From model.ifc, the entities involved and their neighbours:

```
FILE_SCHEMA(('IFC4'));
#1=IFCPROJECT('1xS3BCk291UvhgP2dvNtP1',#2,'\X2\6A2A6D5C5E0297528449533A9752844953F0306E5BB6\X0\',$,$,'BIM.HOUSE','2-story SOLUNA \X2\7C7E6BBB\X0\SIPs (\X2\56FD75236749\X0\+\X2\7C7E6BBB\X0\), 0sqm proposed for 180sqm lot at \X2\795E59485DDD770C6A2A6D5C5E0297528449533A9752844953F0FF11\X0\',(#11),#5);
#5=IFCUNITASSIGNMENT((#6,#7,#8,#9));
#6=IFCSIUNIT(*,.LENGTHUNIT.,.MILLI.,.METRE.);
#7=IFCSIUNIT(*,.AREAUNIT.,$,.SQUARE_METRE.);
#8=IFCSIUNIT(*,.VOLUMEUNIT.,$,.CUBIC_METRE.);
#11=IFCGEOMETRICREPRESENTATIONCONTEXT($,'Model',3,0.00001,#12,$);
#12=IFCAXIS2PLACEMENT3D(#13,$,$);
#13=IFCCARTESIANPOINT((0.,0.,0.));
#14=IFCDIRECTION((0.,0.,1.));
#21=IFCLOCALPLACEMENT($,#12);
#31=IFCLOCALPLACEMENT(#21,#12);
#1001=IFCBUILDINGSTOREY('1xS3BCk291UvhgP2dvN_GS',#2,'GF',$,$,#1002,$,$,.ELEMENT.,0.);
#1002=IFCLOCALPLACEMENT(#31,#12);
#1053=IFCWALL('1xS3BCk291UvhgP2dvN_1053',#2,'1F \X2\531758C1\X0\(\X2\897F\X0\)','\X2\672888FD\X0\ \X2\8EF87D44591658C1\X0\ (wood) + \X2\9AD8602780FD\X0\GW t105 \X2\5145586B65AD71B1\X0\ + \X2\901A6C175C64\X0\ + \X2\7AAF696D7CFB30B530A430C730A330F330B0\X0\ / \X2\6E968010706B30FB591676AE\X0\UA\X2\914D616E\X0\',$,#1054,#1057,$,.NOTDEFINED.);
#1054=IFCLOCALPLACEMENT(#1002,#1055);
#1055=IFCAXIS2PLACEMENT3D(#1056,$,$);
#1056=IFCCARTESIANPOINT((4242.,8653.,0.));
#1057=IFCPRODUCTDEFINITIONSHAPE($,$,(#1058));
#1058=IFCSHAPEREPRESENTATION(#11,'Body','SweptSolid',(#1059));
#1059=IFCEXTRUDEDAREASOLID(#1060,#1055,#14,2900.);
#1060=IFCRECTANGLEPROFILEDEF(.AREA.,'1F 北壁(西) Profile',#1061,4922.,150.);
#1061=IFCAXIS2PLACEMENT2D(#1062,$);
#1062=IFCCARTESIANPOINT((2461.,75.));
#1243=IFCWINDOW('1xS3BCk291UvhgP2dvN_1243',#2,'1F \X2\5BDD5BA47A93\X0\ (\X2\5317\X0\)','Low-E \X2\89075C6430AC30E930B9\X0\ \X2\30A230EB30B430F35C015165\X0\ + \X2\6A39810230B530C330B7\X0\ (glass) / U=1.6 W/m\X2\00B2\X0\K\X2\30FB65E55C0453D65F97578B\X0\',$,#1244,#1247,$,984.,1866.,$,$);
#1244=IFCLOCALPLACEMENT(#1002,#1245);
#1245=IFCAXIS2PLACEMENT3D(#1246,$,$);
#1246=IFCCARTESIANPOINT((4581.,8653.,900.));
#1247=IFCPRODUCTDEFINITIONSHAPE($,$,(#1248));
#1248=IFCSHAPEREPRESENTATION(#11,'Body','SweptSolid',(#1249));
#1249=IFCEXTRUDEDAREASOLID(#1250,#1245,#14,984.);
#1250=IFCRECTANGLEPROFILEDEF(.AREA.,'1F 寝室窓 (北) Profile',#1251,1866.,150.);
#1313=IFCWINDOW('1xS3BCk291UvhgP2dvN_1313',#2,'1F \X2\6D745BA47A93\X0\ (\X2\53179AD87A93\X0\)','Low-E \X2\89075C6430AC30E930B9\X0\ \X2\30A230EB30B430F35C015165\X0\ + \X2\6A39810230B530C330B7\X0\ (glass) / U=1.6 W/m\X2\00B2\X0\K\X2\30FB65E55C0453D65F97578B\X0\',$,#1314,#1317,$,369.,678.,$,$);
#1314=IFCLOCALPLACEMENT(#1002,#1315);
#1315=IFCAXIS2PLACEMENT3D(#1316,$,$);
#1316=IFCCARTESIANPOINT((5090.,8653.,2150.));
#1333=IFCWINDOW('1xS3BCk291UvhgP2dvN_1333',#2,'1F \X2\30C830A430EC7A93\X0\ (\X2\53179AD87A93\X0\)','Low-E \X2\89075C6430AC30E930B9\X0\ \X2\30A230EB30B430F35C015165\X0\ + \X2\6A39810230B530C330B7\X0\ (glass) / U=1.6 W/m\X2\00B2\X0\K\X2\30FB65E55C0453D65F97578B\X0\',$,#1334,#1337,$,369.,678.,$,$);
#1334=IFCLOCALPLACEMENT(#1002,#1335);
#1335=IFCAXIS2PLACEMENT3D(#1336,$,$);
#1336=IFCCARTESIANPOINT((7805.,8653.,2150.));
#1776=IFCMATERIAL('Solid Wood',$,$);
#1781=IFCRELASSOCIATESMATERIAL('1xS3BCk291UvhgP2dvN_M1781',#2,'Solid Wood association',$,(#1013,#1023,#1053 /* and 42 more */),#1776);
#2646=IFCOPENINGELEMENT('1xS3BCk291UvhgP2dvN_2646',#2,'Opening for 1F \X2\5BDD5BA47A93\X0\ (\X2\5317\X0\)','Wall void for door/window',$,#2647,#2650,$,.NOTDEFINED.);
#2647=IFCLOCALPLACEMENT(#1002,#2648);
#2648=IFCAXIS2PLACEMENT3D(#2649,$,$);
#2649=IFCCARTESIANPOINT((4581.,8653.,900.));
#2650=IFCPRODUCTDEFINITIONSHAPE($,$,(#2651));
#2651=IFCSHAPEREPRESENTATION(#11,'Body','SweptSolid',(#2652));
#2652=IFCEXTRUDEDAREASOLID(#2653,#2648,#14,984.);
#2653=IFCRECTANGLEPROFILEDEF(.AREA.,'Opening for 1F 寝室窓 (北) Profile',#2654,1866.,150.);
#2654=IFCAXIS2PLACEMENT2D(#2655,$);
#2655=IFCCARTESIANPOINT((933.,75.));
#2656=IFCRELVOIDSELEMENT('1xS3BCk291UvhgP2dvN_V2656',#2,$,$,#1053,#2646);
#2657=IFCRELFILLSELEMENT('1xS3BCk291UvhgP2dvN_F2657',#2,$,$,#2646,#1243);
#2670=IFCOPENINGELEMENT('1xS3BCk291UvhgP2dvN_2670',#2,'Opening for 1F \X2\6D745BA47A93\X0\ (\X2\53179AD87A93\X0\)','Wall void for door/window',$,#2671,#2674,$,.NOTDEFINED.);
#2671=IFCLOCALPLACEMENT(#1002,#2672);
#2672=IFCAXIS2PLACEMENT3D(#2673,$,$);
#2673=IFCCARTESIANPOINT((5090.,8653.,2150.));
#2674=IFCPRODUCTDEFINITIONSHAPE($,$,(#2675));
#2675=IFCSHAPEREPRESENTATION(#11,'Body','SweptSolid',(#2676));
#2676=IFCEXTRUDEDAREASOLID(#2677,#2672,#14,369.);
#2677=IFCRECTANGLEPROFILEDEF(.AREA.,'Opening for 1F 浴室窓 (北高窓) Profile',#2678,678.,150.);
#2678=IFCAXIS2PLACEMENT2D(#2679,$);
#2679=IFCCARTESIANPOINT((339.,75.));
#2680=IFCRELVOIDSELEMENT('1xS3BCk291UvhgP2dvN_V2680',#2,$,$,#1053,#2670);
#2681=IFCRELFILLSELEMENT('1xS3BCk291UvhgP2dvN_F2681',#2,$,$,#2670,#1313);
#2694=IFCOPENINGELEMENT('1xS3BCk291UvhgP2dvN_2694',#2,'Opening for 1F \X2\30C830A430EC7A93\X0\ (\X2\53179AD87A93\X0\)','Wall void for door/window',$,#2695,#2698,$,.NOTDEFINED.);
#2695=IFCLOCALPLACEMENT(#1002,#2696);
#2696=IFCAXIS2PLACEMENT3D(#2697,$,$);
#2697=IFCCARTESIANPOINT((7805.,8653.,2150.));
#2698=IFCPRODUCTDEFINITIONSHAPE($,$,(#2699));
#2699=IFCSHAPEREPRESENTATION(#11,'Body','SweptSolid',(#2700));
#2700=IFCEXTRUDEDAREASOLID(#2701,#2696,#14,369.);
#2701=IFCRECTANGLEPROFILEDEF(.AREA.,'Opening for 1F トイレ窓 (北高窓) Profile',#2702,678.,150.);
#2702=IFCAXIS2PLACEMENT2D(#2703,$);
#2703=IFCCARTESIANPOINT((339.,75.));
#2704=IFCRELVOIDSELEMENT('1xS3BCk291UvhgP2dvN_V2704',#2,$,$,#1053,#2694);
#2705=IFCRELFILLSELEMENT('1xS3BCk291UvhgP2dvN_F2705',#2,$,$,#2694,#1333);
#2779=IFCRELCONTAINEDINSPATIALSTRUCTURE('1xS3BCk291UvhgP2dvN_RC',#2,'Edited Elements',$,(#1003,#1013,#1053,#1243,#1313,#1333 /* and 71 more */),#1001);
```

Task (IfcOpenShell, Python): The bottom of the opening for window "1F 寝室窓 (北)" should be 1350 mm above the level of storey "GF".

```python
import numpy as np
import ifcopenshell
import ifcopenshell.api.geometry
import ifcopenshell.geom
import ifcopenshell.util.element
import ifcopenshell.util.placement
import ifcopenshell.util.shape
import ifcopenshell.util.unit

model = ifcopenshell.open("model.ifc")
unit_scale = ifcopenshell.util.unit.calculate_unit_scale(model)

window = model.by_guid("1xS3BCk291UvhgP2dvN_1243")
opening = window.FillsVoids[0].RelatingOpeningElement
storey = ifcopenshell.util.element.get_container(window, ifc_class="IfcBuildingStorey")
level = ifcopenshell.util.placement.get_local_placement(storey.ObjectPlacement)[2, 3]

# The opening's origin need not be at the sill, so measure its lowest point.
shape = ifcopenshell.geom.create_shape(ifcopenshell.geom.settings(), opening)
bottom = ifcopenshell.util.shape.get_shape_bottom_elevation(shape, shape.geometry) / unit_scale
dz = level + 1.35 / unit_scale - bottom

shift = np.array([0.0, 0.0, dz])
# The window is not placed relative to its opening, so move both.
for product in (opening, window):
    matrix = ifcopenshell.util.placement.get_local_placement(product.ObjectPlacement)
    matrix[:3, 3] += shift
    ifcopenshell.api.geometry.edit_object_placement(model, product=product, matrix=matrix, is_si=False)

print(f"moved by {dz * unit_scale:+.3f} m")

model.write("model_rev.ifc")
```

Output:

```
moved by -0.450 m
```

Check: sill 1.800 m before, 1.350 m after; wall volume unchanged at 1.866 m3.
